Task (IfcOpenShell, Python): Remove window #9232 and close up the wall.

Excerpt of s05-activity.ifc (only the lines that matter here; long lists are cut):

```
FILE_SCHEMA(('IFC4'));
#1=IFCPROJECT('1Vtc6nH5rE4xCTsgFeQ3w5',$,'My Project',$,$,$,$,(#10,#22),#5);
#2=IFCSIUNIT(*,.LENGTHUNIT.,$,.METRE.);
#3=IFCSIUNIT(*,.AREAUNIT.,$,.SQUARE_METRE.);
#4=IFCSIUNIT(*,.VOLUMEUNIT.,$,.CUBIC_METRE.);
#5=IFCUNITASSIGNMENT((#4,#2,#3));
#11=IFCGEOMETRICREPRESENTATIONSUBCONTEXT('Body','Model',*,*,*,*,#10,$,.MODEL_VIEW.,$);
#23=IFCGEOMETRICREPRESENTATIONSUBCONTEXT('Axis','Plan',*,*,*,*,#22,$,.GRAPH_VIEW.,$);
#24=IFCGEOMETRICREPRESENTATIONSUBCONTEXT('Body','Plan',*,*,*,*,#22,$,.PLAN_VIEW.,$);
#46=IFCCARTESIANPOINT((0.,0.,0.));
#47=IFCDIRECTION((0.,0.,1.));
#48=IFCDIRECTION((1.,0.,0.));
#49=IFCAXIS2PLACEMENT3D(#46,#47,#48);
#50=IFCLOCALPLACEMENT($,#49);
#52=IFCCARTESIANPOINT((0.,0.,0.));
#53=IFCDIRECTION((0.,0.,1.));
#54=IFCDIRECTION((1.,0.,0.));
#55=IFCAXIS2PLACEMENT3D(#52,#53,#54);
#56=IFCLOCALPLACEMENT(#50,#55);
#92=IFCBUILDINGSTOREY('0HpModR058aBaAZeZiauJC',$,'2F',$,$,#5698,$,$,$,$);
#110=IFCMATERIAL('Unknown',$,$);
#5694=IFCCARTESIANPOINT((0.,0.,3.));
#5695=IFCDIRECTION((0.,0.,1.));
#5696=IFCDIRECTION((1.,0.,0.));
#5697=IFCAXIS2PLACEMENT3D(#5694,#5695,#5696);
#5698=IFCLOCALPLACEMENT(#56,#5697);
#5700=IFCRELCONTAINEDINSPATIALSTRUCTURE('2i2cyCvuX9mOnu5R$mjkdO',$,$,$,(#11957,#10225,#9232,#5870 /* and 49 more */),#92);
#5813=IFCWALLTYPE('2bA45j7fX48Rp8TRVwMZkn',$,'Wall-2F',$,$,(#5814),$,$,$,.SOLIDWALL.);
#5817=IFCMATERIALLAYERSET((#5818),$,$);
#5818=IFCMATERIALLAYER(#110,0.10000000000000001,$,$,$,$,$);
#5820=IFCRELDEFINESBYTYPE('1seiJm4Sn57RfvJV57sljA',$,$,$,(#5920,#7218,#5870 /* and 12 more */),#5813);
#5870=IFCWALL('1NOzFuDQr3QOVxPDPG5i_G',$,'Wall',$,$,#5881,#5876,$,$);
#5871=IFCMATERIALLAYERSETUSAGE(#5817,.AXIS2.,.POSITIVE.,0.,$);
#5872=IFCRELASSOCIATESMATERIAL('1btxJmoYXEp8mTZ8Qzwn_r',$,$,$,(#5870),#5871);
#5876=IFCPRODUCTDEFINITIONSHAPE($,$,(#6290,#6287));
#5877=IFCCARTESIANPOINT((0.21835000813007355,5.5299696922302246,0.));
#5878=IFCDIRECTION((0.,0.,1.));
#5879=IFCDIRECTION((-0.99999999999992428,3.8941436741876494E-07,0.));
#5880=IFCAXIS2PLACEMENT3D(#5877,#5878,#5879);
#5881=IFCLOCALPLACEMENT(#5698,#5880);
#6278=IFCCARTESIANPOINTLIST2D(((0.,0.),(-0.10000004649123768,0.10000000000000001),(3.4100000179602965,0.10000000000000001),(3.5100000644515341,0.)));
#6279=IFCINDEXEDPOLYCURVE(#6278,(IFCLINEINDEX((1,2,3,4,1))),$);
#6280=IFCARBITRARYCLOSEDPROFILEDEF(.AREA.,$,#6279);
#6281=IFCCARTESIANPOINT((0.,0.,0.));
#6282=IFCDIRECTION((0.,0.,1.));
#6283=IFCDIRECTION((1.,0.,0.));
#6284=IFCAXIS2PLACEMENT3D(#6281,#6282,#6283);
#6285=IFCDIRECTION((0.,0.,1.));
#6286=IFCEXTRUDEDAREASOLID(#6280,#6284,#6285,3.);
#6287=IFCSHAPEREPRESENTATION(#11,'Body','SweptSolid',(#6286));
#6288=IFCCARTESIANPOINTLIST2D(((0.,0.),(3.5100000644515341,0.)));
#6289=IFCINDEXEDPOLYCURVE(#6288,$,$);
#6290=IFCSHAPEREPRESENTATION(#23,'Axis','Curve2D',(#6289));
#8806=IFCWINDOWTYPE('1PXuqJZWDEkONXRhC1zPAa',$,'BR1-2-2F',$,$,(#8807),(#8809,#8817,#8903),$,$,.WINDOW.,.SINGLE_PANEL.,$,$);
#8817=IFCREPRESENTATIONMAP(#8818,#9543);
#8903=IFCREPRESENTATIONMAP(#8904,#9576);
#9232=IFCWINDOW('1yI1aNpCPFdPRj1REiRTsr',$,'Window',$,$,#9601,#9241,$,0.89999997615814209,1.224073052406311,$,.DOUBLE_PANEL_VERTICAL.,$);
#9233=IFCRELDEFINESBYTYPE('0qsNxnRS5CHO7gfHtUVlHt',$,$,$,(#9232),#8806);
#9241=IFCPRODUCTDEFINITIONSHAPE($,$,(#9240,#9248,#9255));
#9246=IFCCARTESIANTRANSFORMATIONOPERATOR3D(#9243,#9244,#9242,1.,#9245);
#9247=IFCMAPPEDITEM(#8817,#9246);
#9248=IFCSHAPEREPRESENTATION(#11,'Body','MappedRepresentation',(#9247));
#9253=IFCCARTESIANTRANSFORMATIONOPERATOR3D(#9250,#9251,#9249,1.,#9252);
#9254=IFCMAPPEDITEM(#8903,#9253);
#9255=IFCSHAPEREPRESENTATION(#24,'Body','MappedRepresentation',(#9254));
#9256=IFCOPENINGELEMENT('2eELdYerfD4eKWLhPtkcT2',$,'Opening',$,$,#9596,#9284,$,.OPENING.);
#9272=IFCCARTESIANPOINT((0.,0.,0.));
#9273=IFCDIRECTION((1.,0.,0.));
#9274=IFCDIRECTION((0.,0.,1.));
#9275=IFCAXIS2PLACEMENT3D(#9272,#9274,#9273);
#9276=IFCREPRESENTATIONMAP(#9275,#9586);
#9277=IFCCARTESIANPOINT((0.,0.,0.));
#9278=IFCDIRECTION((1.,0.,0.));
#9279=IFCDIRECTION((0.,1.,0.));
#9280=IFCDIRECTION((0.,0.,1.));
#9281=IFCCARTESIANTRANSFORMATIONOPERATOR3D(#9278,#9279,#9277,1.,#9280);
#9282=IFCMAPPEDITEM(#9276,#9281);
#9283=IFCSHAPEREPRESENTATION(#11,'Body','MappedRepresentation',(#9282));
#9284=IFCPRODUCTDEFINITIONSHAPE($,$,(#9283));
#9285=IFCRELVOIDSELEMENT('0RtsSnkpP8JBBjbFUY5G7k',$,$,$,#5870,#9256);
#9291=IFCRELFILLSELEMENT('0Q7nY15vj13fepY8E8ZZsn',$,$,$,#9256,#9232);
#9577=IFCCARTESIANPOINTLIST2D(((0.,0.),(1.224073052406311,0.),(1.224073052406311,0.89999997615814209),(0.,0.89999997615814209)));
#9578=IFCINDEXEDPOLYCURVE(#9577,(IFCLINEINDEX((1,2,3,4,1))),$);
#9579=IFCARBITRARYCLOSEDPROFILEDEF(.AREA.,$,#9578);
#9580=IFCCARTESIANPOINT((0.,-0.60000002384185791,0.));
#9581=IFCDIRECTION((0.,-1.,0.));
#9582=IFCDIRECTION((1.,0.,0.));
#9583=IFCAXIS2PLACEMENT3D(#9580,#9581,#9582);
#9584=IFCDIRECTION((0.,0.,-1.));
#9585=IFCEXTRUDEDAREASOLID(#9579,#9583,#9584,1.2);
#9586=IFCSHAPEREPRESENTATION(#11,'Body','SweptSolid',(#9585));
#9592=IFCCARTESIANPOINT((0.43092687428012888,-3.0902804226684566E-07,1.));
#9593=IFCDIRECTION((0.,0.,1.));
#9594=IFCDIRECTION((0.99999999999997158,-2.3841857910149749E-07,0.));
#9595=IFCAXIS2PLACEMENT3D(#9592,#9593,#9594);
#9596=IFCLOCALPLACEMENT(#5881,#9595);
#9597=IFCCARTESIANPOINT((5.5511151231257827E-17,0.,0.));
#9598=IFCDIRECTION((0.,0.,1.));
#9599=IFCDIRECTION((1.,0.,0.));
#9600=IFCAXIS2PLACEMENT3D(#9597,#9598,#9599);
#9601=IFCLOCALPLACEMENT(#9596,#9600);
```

```python
import ifcopenshell
import ifcopenshell.api.feature
import ifcopenshell.api.root
import ifcopenshell.geom
import ifcopenshell.util.shape

model = ifcopenshell.open("s05-activity.ifc")
settings = ifcopenshell.geom.settings()


def volume(element):
    """Net volume in cubic metres, openings subtracted."""
    shape = ifcopenshell.geom.create_shape(settings, element)
    return ifcopenshell.util.shape.get_volume(shape.geometry)


window = model.by_guid("1yI1aNpCPFdPRj1REiRTsr")
opening = window.FillsVoids[0].RelatingOpeningElement
wall = opening.VoidsElements[0].RelatingBuildingElement
before = volume(wall)

ifcopenshell.api.root.remove_product(model, product=window)
ifcopenshell.api.feature.remove_feature(model, feature=opening)

after = volume(wall)

print(f"wall volume {before:.3f} -> {after:.3f} m3")

model.write("s05-activity_rev.ifc")
```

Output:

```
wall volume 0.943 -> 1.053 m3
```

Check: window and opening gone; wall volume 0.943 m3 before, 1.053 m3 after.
